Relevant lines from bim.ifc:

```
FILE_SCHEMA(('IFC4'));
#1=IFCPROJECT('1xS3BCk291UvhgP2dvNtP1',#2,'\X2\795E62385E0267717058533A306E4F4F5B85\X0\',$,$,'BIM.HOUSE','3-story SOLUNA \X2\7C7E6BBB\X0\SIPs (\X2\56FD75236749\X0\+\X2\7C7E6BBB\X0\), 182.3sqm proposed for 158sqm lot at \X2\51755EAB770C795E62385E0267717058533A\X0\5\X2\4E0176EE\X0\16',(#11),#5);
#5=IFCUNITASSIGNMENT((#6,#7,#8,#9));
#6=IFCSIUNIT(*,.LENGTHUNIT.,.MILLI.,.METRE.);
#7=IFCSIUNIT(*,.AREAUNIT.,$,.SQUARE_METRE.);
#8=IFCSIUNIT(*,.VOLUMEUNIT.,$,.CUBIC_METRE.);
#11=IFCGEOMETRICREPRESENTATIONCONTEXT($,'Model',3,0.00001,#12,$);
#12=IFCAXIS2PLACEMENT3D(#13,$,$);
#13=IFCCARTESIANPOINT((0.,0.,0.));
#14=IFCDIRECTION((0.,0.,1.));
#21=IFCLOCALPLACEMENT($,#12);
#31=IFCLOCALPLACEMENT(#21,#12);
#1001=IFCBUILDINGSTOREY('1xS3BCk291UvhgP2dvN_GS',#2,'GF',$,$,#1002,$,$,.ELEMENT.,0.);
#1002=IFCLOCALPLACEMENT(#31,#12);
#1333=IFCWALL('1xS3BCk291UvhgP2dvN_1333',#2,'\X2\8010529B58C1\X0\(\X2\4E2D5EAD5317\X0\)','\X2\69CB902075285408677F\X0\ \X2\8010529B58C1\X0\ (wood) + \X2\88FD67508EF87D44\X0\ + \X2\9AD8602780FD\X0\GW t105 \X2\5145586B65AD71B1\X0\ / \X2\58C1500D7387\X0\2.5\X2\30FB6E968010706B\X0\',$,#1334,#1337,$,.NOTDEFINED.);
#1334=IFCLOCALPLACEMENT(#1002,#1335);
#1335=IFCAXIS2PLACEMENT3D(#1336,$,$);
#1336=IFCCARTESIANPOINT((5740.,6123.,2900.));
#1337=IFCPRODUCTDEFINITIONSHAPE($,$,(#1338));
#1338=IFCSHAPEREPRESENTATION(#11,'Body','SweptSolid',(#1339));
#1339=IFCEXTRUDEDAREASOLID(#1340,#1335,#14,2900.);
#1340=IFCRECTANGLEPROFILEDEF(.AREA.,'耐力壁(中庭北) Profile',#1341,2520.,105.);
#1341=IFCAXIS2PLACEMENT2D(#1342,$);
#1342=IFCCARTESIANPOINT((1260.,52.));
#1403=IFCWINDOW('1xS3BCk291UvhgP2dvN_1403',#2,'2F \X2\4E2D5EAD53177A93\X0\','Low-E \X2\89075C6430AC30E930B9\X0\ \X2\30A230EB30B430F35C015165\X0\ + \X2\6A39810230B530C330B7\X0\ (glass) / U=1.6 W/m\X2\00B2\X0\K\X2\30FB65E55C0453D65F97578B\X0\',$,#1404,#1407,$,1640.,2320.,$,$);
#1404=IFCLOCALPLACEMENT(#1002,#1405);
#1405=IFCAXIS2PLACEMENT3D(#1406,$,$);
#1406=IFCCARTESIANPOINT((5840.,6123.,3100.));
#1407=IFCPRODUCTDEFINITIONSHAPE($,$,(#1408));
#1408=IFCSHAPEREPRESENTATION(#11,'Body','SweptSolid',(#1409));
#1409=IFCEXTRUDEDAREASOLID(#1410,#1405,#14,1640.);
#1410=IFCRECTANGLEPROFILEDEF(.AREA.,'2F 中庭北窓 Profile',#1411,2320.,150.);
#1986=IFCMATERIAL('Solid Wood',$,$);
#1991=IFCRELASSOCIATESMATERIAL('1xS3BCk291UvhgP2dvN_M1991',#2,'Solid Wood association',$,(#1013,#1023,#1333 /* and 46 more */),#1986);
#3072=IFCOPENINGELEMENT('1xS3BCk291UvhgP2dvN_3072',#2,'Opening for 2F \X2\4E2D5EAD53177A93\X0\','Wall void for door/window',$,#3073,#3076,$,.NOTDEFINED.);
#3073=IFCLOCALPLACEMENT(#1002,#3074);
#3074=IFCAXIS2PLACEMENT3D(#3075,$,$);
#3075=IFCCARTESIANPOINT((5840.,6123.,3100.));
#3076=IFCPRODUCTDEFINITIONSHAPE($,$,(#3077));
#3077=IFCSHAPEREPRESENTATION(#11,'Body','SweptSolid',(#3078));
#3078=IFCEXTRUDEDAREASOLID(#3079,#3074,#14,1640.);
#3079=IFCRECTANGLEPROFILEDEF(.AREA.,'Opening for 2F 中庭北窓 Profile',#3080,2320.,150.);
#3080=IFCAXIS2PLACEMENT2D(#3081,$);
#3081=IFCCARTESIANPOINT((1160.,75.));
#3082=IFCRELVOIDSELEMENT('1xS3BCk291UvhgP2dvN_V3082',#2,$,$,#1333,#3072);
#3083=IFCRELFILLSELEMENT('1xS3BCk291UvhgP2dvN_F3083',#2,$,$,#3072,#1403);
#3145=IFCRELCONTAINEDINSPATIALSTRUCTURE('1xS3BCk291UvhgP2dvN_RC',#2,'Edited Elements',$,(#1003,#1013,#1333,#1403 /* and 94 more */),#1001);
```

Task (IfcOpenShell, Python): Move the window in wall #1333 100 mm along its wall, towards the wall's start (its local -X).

```python
import ifcopenshell
import ifcopenshell.api.geometry
import ifcopenshell.util.placement
import ifcopenshell.util.unit

model = ifcopenshell.open("bim.ifc")
unit_scale = ifcopenshell.util.unit.calculate_unit_scale(model)

window = model.by_id(1403)
opening = window.FillsVoids[0].RelatingOpeningElement
wall = opening.VoidsElements[0].RelatingBuildingElement

wall_matrix = ifcopenshell.util.placement.get_local_placement(wall.ObjectPlacement)
shift = wall_matrix[:3, 0] * -0.1 / unit_scale
before = ifcopenshell.util.placement.get_local_placement(window.ObjectPlacement)[:3, 3].copy()

# The window is not placed relative to its opening, so move both.
for product in (opening, window):
    matrix = ifcopenshell.util.placement.get_local_placement(product.ObjectPlacement)
    matrix[:3, 3] += shift
    ifcopenshell.api.geometry.edit_object_placement(model, product=product, matrix=matrix, is_si=False)

after = ifcopenshell.util.placement.get_local_placement(window.ObjectPlacement)[:3, 3]
print("window moved by", (after - before).round(3) + 0.0)

model.write("bim_updated.ifc")
```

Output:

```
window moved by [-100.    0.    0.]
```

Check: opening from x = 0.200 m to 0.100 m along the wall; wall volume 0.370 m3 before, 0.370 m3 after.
